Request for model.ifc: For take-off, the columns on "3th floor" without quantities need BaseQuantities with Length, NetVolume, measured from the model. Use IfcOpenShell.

First a look at what the model holds.

```python
import ifcopenshell
import ifcopenshell.util.element
import ifcopenshell.util.unit

model = ifcopenshell.open("model.ifc")
print(model.schema)
for unit_type in ("LENGTHUNIT", "AREAUNIT", "VOLUMEUNIT"):
    print(unit_type, ifcopenshell.util.unit.calculate_unit_scale(model, unit_type))
storey = next(s for s in model.by_type("IfcBuildingStorey") if s.Name == "3th floor")
columns = [e for e in ifcopenshell.util.element.get_decomposition(storey) if e.is_a("IfcColumn")]
for e in sorted(columns, key=lambda e: e.id()):
    print(e.id(), e.is_a(), e.Name, list(ifcopenshell.util.element.get_psets(e, qtos_only=True)), sep=" | ")
```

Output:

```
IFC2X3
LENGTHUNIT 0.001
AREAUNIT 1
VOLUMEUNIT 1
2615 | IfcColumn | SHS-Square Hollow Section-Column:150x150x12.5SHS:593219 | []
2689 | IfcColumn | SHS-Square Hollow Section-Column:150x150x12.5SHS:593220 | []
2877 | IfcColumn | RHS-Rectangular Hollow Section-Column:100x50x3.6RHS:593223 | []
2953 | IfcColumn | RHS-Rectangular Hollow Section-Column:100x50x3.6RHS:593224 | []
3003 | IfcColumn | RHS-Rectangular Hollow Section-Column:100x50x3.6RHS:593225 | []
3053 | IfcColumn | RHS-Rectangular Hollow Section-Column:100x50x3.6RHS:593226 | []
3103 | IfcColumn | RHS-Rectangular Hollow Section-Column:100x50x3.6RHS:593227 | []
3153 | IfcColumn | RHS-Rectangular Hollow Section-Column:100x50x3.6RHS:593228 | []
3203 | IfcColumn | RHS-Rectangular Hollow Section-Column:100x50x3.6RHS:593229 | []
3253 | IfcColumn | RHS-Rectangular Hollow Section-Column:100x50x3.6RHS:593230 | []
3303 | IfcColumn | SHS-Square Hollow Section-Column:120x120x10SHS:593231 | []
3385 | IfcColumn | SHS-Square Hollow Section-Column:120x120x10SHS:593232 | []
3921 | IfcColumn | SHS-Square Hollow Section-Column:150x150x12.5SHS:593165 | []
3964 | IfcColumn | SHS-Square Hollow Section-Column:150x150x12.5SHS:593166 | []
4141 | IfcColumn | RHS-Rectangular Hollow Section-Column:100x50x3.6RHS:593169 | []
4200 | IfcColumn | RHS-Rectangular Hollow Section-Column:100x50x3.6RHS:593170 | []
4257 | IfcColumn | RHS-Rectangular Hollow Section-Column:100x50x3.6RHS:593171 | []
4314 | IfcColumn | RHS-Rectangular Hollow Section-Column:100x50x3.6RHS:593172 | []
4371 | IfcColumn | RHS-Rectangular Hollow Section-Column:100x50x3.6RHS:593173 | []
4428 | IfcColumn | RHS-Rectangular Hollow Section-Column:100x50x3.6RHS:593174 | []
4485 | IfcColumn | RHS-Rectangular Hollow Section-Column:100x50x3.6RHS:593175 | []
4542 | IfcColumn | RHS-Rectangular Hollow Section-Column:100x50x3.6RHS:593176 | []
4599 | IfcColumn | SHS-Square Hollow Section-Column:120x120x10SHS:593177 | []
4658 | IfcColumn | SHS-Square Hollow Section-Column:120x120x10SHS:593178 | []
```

```python
import ifcopenshell
import ifcopenshell.api.pset
import ifcopenshell.geom
import ifcopenshell.util.element
import ifcopenshell.util.shape
import ifcopenshell.util.unit

model = ifcopenshell.open("model.ifc")
unit_scale = ifcopenshell.util.unit.calculate_unit_scale(model)
volume_scale = ifcopenshell.util.unit.calculate_unit_scale(model, "VOLUMEUNIT")
settings = ifcopenshell.geom.settings()

storey = next(s for s in model.by_type("IfcBuildingStorey") if s.Name == "3th floor")
columns = [e for e in ifcopenshell.util.element.get_decomposition(storey) if e.is_a("IfcColumn")]

for e in sorted(columns, key=lambda e: e.id()):
    if ifcopenshell.util.element.get_psets(e, qtos_only=True, should_inherit=False):
        continue
    # Geometry comes back in metres, in the element's own axes.
    shape = ifcopenshell.geom.create_shape(settings, e)
    values = {
        "Length": ifcopenshell.util.shape.get_z(shape.geometry) / unit_scale,
        "NetVolume": ifcopenshell.util.shape.get_volume(shape.geometry) / volume_scale,
    }
    qto = ifcopenshell.api.pset.add_qto(model, product=e, name="BaseQuantities")
    ifcopenshell.api.pset.edit_qto(model, qto=qto, properties=values)
    print(e.id(), {k: round(v, 3) for k, v in values.items()})

model.write("model_updated.ifc")
```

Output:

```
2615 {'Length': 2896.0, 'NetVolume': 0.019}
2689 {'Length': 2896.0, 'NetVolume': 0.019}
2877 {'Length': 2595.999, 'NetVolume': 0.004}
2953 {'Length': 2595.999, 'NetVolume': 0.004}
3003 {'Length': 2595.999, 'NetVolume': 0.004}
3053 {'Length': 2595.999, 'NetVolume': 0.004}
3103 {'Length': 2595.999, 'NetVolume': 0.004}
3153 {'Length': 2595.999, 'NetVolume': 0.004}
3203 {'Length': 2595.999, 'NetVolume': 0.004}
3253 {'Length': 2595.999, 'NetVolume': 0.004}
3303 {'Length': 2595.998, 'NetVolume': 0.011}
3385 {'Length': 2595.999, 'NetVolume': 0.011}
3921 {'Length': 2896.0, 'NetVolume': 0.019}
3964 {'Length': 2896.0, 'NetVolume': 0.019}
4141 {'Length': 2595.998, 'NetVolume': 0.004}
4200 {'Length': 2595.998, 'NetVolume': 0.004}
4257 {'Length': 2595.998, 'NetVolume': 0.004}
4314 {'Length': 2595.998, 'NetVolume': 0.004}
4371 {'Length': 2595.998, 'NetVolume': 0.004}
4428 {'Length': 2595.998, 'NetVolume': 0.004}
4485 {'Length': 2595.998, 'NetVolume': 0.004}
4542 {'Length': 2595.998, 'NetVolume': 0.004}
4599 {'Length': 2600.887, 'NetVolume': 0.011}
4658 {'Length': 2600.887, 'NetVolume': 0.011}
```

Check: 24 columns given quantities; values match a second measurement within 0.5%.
